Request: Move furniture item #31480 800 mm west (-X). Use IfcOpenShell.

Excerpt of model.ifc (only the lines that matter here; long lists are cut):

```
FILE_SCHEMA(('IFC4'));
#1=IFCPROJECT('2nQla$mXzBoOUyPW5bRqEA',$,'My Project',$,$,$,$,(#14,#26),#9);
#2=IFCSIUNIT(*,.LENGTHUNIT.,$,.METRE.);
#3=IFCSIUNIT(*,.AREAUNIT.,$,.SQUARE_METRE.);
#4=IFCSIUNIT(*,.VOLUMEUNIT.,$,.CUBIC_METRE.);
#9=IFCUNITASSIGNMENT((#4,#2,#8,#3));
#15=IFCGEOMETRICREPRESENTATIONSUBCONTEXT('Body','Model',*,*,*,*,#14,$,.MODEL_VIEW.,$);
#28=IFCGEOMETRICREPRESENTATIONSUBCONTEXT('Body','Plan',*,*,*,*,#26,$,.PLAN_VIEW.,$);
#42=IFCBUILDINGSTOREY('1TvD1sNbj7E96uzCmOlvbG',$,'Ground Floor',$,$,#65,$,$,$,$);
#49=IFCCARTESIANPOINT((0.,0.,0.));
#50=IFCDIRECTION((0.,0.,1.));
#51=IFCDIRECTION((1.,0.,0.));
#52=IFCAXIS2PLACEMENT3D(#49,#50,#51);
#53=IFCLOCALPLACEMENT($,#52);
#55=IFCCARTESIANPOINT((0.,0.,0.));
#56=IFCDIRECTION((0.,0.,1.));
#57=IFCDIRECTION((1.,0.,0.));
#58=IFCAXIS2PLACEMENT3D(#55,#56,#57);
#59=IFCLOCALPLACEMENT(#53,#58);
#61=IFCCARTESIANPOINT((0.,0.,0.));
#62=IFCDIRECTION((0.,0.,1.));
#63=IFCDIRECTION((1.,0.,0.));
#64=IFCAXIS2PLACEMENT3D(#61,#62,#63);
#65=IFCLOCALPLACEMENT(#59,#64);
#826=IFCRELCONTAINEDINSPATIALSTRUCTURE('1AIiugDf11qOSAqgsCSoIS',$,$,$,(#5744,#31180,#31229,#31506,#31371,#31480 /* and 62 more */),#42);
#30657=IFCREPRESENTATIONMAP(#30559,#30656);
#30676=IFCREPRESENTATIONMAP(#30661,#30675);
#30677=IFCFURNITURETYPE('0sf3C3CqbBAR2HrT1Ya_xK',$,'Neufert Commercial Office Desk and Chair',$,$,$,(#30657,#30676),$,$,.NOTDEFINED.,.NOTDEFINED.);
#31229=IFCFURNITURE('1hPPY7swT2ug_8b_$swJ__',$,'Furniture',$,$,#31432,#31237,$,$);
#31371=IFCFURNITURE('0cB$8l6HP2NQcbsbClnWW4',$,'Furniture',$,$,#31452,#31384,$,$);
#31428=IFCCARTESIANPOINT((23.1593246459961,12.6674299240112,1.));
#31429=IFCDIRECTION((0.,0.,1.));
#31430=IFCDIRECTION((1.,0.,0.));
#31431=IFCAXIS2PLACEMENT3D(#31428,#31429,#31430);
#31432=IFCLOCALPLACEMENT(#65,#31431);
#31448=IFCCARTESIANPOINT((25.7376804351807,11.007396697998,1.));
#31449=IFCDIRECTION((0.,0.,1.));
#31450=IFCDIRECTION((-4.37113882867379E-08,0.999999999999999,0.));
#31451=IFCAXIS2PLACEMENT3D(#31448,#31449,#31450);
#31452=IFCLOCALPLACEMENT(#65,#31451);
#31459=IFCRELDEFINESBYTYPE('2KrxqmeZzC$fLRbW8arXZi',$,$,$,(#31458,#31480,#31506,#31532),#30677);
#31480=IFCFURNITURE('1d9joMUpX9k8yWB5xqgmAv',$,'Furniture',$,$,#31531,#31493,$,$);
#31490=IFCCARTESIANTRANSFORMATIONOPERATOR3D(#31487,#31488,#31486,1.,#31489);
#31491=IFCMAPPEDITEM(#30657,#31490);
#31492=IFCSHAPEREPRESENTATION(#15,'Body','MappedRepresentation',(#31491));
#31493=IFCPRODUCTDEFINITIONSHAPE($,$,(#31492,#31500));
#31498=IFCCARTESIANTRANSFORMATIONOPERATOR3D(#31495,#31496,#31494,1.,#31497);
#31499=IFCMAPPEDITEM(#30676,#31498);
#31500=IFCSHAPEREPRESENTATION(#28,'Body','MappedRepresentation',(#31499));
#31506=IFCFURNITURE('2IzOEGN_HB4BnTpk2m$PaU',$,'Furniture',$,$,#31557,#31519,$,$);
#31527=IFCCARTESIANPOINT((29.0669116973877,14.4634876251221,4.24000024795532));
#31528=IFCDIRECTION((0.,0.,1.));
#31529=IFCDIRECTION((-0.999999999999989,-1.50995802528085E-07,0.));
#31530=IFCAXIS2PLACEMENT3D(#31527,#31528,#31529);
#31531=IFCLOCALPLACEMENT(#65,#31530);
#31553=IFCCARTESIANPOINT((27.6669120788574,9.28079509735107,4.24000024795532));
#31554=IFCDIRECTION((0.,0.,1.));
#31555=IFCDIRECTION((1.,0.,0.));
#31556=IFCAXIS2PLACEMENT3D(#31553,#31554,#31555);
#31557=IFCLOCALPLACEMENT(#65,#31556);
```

```python
import ifcopenshell
import ifcopenshell.api.geometry
import ifcopenshell.util.placement

model = ifcopenshell.open("model.ifc")

item = model.by_id(31480)
matrix = ifcopenshell.util.placement.get_local_placement(item.ObjectPlacement)
matrix[0, 3] -= 0.8
ifcopenshell.api.geometry.edit_object_placement(model, product=item, matrix=matrix, is_si=False)

print(ifcopenshell.util.placement.get_local_placement(item.ObjectPlacement).round(3) + 0.0)

model.write("model_rev.ifc")
```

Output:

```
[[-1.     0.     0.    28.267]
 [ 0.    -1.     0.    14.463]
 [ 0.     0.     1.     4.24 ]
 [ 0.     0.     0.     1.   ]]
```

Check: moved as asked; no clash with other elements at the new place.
